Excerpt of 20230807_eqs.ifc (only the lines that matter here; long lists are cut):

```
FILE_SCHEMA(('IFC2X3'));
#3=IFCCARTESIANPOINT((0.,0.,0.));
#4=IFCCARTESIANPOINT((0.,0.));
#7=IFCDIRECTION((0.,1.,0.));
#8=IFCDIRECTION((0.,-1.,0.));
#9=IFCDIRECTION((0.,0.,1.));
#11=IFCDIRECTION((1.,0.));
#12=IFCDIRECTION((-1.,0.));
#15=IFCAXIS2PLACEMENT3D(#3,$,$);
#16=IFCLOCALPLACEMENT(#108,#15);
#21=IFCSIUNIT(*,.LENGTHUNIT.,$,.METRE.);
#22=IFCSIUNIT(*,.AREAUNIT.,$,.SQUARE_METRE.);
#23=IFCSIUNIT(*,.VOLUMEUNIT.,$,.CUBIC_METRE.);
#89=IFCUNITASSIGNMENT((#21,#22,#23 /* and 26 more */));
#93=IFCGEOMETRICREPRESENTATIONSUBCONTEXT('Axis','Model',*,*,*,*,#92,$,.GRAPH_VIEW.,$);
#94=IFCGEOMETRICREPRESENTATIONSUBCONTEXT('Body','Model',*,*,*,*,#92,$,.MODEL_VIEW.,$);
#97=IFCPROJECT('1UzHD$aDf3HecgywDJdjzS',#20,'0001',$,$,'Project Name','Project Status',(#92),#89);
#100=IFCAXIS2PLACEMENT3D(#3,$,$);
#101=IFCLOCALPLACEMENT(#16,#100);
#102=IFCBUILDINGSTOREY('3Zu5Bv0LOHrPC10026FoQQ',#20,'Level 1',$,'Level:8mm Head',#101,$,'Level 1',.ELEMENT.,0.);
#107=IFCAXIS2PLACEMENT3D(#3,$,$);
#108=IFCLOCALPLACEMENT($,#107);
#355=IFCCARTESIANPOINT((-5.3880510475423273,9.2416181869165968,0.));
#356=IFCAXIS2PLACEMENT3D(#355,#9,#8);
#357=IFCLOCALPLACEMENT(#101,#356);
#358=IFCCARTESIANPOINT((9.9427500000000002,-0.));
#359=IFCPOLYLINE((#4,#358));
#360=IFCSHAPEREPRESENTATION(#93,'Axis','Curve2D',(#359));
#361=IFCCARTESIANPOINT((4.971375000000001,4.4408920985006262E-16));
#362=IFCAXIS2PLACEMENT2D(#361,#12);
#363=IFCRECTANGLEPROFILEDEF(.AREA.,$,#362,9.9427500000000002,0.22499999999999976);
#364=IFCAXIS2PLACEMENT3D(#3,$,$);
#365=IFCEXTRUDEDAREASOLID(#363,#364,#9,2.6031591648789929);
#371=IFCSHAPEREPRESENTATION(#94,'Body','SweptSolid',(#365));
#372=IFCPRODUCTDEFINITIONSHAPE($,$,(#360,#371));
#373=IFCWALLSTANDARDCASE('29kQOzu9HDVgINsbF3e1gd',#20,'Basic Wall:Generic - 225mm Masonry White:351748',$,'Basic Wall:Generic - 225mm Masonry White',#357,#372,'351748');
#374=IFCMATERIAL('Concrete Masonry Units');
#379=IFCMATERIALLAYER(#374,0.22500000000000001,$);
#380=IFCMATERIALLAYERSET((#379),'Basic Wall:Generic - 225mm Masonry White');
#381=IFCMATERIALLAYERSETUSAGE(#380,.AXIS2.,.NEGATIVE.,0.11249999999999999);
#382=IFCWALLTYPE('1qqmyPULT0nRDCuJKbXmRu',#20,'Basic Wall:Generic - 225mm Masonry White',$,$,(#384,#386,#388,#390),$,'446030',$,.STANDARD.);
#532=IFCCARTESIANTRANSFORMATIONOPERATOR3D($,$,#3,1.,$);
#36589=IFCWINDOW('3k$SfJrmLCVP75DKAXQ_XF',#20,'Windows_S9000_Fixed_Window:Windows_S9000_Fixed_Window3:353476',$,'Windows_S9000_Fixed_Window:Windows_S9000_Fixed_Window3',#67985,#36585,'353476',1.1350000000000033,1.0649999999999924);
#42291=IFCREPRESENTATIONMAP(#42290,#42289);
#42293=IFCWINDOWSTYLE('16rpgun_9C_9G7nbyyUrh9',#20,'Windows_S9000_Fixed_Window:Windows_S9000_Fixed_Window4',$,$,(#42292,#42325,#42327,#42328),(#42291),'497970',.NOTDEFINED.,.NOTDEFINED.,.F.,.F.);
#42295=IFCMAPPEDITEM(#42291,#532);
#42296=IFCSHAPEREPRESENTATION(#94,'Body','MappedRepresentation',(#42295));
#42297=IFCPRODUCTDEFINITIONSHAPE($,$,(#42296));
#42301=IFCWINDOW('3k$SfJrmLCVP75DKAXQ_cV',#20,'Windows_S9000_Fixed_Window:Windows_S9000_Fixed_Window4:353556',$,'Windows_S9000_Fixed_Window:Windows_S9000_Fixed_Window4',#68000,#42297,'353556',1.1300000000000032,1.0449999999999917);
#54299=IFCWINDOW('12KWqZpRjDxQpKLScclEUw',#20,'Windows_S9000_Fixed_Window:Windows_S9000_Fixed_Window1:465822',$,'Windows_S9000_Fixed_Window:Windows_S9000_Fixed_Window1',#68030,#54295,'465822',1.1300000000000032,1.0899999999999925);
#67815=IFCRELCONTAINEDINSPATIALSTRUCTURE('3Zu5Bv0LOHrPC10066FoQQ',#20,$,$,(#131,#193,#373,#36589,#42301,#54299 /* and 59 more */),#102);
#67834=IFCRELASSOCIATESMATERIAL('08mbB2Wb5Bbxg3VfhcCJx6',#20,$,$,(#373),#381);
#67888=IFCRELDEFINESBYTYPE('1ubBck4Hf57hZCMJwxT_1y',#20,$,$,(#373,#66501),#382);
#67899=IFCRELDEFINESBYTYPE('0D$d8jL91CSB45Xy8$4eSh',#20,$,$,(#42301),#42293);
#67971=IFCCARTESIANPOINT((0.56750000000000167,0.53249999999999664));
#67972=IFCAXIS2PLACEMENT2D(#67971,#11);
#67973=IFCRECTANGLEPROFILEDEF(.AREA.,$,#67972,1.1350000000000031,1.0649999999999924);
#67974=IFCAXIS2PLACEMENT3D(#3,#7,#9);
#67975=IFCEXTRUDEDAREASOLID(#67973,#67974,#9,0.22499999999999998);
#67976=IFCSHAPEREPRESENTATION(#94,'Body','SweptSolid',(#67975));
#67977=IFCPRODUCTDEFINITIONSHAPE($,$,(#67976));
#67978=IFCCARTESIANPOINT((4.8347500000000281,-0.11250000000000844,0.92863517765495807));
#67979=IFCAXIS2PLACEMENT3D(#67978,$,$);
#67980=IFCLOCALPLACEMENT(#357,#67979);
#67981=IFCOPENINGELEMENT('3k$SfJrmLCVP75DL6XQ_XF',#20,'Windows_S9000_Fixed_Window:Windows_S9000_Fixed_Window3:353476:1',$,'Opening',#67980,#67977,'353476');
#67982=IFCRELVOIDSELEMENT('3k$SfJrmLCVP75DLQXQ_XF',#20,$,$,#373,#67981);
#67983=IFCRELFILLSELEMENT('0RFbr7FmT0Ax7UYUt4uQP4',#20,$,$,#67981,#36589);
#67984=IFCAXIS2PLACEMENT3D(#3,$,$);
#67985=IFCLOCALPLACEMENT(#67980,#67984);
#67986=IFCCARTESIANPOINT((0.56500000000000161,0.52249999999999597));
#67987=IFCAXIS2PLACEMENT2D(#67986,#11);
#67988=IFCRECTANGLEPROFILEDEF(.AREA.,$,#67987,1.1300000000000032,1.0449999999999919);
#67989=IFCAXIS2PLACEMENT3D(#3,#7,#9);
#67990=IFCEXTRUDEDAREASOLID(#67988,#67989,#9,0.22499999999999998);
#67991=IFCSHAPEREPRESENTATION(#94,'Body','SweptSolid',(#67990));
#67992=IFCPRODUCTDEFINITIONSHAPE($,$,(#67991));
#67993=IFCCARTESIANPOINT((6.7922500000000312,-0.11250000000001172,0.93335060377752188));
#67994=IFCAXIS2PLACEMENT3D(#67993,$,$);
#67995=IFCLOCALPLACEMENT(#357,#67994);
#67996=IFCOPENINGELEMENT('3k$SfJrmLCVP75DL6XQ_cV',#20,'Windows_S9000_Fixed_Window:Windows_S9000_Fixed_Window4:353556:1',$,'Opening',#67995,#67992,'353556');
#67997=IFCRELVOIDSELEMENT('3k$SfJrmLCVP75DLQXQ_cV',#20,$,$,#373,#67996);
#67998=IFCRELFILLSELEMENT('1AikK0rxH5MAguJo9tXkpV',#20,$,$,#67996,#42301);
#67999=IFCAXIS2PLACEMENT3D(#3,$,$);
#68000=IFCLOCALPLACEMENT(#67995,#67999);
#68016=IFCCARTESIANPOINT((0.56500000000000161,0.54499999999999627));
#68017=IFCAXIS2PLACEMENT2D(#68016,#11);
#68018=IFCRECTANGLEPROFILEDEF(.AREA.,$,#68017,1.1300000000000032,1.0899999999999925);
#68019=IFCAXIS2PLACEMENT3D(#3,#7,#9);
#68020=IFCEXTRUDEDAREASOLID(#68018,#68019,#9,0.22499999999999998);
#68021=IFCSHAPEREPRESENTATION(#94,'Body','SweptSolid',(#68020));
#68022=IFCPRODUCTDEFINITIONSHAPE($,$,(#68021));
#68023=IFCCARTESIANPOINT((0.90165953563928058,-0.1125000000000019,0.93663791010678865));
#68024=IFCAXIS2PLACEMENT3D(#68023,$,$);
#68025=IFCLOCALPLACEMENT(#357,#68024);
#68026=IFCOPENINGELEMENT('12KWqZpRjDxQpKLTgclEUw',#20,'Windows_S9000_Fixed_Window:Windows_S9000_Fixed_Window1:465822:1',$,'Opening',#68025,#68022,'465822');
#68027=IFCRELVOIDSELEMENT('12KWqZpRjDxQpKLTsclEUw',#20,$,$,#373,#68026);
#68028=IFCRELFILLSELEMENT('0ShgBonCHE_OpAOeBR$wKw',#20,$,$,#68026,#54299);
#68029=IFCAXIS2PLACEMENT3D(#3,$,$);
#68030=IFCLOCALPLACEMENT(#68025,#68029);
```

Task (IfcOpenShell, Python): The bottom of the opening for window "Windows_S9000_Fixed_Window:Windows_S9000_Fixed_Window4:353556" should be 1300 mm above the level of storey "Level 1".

```python
import numpy as np
import ifcopenshell
import ifcopenshell.api.geometry
import ifcopenshell.geom
import ifcopenshell.util.element
import ifcopenshell.util.placement
import ifcopenshell.util.shape
import ifcopenshell.util.unit

model = ifcopenshell.open("20230807_eqs.ifc")
unit_scale = ifcopenshell.util.unit.calculate_unit_scale(model)

window = model.by_guid("3k$SfJrmLCVP75DKAXQ_cV")
opening = window.FillsVoids[0].RelatingOpeningElement
storey = ifcopenshell.util.element.get_container(window, ifc_class="IfcBuildingStorey")
level = ifcopenshell.util.placement.get_local_placement(storey.ObjectPlacement)[2, 3]

# The opening's origin need not be at the sill, so measure its lowest point.
shape = ifcopenshell.geom.create_shape(ifcopenshell.geom.settings(), opening)
bottom = ifcopenshell.util.shape.get_shape_bottom_elevation(shape, shape.geometry) / unit_scale
dz = level + 1.3 / unit_scale - bottom

shift = np.array([0.0, 0.0, dz])
# The window is placed relative to its opening, so it follows when the opening moves.
matrix = ifcopenshell.util.placement.get_local_placement(opening.ObjectPlacement)
matrix[:3, 3] += shift
ifcopenshell.api.geometry.edit_object_placement(
    model, product=opening, matrix=matrix, is_si=False, should_transform_children=True
)

print(f"moved by {dz * unit_scale:+.3f} m")

model.write("20230807_eqs_v2.ifc")
```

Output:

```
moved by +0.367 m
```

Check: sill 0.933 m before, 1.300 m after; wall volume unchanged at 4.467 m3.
